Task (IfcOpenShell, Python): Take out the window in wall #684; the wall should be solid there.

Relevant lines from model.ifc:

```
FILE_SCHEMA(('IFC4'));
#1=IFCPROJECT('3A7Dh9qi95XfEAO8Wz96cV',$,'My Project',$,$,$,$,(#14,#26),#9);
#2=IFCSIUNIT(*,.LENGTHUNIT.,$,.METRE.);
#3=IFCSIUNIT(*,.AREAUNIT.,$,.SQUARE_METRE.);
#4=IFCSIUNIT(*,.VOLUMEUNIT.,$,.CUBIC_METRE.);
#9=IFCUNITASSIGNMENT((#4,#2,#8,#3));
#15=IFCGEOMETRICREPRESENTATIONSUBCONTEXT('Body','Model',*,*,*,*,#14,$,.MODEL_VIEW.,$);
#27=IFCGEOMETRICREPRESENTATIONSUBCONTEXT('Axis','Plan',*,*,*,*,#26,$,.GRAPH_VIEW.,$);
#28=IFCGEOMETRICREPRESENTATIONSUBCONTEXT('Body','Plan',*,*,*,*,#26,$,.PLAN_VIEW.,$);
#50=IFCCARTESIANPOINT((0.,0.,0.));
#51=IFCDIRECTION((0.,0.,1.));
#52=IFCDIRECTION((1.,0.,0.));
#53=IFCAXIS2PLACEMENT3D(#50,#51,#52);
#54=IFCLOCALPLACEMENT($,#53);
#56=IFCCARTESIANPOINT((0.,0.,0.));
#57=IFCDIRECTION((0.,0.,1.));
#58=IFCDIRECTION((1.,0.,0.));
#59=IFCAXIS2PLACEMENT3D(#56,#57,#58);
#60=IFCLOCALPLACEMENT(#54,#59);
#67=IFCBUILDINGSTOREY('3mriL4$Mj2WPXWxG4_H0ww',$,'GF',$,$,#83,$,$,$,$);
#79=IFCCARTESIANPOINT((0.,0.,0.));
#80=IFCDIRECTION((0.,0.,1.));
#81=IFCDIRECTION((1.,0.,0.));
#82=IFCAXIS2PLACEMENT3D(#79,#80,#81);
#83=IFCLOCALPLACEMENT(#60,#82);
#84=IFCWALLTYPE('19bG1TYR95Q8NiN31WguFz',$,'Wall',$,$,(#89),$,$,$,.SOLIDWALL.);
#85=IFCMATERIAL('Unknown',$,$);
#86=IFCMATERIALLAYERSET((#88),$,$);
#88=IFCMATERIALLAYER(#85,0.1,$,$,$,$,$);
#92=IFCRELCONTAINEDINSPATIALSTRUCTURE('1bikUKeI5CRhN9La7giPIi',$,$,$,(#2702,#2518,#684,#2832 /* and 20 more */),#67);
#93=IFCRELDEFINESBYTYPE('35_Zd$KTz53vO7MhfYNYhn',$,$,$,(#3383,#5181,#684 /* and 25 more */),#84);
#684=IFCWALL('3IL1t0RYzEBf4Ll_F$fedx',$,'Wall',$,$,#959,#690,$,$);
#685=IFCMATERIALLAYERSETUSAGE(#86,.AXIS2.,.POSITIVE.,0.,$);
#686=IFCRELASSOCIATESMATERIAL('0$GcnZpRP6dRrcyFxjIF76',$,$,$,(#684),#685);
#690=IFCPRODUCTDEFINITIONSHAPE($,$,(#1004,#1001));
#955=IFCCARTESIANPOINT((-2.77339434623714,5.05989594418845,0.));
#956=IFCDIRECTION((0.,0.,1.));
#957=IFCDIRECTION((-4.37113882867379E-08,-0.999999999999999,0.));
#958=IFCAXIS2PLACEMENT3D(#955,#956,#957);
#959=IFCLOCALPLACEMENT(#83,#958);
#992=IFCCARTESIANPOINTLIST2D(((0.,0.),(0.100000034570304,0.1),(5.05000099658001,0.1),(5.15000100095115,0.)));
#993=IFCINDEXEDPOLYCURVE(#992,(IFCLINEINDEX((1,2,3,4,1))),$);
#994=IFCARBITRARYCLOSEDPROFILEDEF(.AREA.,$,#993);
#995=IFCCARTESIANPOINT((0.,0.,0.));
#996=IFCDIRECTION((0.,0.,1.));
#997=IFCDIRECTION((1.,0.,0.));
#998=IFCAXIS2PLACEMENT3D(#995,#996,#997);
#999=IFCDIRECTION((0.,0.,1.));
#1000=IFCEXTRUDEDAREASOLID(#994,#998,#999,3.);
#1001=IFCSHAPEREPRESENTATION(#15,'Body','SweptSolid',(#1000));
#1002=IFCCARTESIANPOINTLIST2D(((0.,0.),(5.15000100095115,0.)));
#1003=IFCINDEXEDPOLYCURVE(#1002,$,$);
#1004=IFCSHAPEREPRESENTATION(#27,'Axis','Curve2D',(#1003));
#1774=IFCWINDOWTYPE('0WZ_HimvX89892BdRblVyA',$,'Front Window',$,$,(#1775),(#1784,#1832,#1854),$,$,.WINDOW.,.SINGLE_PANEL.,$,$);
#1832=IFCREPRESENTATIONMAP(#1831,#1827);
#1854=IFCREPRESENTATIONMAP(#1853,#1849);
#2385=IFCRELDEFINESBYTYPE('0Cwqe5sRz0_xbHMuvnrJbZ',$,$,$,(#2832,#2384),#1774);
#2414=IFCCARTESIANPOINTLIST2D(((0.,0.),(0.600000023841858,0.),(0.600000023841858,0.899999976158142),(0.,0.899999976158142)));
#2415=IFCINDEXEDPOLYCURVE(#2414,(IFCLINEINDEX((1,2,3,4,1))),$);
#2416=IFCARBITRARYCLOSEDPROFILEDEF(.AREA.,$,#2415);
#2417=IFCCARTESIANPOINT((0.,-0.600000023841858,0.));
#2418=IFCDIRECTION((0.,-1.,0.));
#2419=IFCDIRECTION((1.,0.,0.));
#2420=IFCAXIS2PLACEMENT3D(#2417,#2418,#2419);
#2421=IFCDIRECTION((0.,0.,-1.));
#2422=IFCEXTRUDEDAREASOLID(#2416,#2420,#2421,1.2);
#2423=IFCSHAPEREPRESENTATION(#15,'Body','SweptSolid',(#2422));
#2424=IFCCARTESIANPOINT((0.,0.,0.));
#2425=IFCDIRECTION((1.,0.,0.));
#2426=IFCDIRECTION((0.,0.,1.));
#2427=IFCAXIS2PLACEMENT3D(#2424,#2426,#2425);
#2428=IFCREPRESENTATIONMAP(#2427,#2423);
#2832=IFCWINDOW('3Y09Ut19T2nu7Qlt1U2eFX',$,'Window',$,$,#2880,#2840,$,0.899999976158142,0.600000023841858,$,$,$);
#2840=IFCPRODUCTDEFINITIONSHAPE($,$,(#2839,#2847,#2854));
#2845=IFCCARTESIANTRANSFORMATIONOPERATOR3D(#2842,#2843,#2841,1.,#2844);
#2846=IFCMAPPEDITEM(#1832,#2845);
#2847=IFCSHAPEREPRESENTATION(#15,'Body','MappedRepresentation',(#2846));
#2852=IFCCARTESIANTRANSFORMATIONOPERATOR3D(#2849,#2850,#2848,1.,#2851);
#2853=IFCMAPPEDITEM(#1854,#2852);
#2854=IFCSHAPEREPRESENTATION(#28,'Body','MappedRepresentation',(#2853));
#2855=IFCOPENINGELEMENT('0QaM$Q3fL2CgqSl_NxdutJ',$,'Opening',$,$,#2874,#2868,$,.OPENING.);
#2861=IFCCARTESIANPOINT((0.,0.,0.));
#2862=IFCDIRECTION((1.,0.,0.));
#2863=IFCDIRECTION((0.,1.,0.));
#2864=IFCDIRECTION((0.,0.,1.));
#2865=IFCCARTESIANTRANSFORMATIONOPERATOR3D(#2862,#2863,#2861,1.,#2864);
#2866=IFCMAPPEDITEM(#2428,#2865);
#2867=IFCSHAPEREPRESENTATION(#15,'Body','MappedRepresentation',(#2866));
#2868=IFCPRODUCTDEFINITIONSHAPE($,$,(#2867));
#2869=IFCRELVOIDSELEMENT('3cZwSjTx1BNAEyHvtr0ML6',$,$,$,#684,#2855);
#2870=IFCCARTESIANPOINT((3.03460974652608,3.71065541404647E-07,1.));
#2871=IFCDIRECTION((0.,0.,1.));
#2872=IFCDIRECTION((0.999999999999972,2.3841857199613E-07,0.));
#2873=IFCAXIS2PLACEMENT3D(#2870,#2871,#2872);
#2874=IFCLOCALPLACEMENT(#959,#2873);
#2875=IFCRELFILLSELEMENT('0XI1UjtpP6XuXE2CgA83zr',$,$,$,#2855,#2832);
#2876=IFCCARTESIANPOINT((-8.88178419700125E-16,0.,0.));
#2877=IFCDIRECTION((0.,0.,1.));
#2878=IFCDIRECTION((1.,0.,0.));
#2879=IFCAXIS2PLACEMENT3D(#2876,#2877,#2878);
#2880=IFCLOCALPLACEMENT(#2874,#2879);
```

```python
import ifcopenshell
import ifcopenshell.api.feature
import ifcopenshell.api.root
import ifcopenshell.geom
import ifcopenshell.util.shape

model = ifcopenshell.open("model.ifc")
settings = ifcopenshell.geom.settings()


def volume(element):
    """Net volume in cubic metres, openings subtracted."""
    shape = ifcopenshell.geom.create_shape(settings, element)
    return ifcopenshell.util.shape.get_volume(shape.geometry)


window = model.by_guid("3Y09Ut19T2nu7Qlt1U2eFX")
opening = window.FillsVoids[0].RelatingOpeningElement
wall = opening.VoidsElements[0].RelatingBuildingElement
before = volume(wall)

ifcopenshell.api.root.remove_product(model, product=window)
ifcopenshell.api.feature.remove_feature(model, feature=opening)

after = volume(wall)

print(f"wall volume {before:.3f} -> {after:.3f} m3")

model.write("model_updated.ifc")
```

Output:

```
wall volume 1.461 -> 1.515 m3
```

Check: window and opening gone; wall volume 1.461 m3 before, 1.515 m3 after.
